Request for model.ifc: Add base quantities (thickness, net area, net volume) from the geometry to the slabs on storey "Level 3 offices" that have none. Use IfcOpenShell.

First a look at what the model holds.

```python
import ifcopenshell
import ifcopenshell.util.element
import ifcopenshell.util.unit

model = ifcopenshell.open("model.ifc")
print(model.schema)
for unit_type in ("LENGTHUNIT", "AREAUNIT", "VOLUMEUNIT"):
    print(unit_type, ifcopenshell.util.unit.calculate_unit_scale(model, unit_type))
storey = next(s for s in model.by_type("IfcBuildingStorey") if s.Name == "Level 3 offices")
slabs = [e for e in ifcopenshell.util.element.get_decomposition(storey) if e.is_a("IfcSlab")]
for e in sorted(slabs, key=lambda e: e.id()):
    print(e.id(), e.is_a(), e.Name, list(ifcopenshell.util.element.get_psets(e, qtos_only=True)), sep=" | ")
```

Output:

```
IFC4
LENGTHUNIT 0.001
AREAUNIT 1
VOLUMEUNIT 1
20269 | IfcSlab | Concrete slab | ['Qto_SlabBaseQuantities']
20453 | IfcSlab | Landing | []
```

```python
import ifcopenshell
import ifcopenshell.api.pset
import ifcopenshell.geom
import ifcopenshell.util.element
import ifcopenshell.util.shape
import ifcopenshell.util.unit

model = ifcopenshell.open("model.ifc")
unit_scale = ifcopenshell.util.unit.calculate_unit_scale(model)
area_scale = ifcopenshell.util.unit.calculate_unit_scale(model, "AREAUNIT")
volume_scale = ifcopenshell.util.unit.calculate_unit_scale(model, "VOLUMEUNIT")
settings = ifcopenshell.geom.settings()

storey = next(s for s in model.by_type("IfcBuildingStorey") if s.Name == "Level 3 offices")
slabs = [e for e in ifcopenshell.util.element.get_decomposition(storey) if e.is_a("IfcSlab")]

for e in sorted(slabs, key=lambda e: e.id()):
    if ifcopenshell.util.element.get_psets(e, qtos_only=True, should_inherit=False):
        continue
    # Geometry comes back in metres, in the element's own axes.
    shape = ifcopenshell.geom.create_shape(settings, e)
    values = {
        "Width": ifcopenshell.util.shape.get_z(shape.geometry) / unit_scale,
        "NetArea": ifcopenshell.util.shape.get_footprint_area(shape.geometry) / area_scale,
        "NetVolume": ifcopenshell.util.shape.get_volume(shape.geometry) / volume_scale,
    }
    qto = ifcopenshell.api.pset.add_qto(model, product=e, name="Qto_SlabBaseQuantities")
    ifcopenshell.api.pset.edit_qto(model, qto=qto, properties=values)
    print(e.id(), {k: round(v, 3) for k, v in values.items()})

model.write("model_v2.ifc")
```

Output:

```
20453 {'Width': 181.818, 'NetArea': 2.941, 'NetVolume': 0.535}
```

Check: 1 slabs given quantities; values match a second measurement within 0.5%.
